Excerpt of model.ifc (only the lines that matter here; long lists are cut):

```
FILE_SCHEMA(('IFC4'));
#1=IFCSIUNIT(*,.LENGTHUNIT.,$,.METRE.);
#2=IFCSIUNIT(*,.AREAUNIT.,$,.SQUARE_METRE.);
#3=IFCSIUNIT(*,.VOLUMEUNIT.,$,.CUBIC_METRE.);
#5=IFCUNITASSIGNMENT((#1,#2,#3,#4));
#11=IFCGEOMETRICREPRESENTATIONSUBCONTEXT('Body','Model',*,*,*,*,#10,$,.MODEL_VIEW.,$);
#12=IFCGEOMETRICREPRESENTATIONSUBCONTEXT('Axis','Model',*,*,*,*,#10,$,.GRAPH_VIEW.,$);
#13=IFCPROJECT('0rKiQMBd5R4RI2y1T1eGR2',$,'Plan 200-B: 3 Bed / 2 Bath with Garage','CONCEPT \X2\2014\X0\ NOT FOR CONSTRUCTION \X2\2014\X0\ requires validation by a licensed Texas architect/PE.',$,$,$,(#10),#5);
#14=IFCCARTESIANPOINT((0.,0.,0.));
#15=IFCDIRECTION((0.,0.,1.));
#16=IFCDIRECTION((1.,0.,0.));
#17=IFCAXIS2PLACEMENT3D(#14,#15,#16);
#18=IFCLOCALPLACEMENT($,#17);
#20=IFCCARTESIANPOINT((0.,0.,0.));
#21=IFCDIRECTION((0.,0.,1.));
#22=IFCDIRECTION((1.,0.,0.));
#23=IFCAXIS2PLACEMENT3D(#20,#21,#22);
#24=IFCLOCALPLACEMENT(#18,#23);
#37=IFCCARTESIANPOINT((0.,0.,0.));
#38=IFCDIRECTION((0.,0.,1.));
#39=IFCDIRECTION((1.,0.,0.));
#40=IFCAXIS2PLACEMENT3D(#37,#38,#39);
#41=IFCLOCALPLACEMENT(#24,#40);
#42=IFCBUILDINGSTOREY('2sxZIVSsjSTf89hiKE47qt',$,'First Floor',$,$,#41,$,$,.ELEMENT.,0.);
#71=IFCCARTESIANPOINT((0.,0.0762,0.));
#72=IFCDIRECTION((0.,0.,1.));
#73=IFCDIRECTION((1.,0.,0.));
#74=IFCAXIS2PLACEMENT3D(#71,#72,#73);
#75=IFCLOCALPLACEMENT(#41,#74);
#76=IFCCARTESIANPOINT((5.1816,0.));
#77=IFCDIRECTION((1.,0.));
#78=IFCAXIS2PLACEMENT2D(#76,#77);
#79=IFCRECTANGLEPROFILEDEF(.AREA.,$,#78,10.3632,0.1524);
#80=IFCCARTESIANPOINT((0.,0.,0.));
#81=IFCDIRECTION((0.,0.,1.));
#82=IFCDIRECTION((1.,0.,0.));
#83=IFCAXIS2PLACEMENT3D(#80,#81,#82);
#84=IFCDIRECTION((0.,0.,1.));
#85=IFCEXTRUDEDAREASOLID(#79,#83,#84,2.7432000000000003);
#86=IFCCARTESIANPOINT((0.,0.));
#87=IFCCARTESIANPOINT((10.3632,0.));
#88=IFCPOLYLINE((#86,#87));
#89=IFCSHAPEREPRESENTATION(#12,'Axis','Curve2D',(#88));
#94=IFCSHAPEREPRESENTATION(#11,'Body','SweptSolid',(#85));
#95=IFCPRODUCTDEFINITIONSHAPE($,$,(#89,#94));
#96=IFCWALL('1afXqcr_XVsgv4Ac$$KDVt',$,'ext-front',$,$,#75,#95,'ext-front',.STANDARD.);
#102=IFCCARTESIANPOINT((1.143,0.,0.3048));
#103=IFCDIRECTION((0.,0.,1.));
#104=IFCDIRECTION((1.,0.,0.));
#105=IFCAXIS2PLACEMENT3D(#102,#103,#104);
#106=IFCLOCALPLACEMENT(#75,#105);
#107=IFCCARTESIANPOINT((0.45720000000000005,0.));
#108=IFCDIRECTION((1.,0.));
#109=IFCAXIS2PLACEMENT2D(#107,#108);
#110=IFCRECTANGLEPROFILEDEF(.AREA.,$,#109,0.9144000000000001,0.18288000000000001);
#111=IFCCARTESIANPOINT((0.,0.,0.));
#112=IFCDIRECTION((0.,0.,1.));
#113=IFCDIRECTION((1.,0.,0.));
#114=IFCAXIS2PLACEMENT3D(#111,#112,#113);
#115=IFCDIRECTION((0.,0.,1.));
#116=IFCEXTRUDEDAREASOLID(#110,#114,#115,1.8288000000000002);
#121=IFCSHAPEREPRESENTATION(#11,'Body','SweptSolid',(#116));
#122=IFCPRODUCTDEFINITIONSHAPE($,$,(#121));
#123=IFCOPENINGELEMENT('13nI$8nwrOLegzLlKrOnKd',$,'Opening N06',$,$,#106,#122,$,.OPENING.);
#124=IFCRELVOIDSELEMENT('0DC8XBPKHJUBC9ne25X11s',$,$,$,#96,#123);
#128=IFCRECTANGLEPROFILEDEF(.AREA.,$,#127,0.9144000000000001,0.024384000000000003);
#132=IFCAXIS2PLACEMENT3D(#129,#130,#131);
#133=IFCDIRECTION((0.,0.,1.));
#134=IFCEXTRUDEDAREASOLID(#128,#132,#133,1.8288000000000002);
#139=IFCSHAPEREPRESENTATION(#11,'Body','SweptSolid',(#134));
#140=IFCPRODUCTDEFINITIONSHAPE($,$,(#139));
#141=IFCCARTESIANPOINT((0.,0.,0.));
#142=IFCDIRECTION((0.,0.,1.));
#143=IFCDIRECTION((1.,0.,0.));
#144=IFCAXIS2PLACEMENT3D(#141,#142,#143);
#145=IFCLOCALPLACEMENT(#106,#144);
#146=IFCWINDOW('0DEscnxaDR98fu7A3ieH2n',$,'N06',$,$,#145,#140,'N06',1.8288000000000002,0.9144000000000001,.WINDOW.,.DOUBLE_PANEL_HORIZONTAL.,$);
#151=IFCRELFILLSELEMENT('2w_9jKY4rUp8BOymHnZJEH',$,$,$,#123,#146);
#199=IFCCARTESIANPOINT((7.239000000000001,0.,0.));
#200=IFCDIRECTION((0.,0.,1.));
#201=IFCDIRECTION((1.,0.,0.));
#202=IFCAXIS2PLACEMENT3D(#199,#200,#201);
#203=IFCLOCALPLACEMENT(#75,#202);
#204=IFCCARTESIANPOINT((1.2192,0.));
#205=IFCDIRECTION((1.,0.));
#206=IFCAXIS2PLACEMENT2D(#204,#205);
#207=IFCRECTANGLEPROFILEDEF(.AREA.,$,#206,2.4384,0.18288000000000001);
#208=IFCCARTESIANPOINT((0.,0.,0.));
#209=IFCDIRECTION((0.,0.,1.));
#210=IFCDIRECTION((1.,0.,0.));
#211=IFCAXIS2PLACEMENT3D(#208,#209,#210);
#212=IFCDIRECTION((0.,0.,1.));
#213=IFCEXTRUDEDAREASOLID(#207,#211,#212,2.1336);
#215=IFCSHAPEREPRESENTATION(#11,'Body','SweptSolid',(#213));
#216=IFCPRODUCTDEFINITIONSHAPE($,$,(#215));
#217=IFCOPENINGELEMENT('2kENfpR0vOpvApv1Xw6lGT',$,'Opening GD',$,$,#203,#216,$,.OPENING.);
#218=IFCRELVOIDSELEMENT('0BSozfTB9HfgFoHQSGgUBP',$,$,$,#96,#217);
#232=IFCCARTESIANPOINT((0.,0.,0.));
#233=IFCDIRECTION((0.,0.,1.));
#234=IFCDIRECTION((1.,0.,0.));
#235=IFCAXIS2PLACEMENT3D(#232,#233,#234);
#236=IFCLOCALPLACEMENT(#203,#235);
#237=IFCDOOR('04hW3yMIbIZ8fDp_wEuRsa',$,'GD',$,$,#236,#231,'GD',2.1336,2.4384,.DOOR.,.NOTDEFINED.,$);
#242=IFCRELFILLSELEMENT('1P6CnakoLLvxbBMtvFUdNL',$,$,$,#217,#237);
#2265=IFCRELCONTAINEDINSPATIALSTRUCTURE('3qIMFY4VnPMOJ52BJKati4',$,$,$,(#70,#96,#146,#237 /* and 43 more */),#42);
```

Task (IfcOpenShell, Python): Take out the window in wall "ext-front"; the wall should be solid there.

```python
import ifcopenshell
import ifcopenshell.api.feature
import ifcopenshell.api.root
import ifcopenshell.geom
import ifcopenshell.util.shape

model = ifcopenshell.open("model.ifc")
settings = ifcopenshell.geom.settings()


def volume(element):
    """Net volume in cubic metres, openings subtracted."""
    shape = ifcopenshell.geom.create_shape(settings, element)
    return ifcopenshell.util.shape.get_volume(shape.geometry)


window = model.by_guid("0DEscnxaDR98fu7A3ieH2n")
opening = window.FillsVoids[0].RelatingOpeningElement
wall = opening.VoidsElements[0].RelatingBuildingElement
before = volume(wall)

ifcopenshell.api.root.remove_product(model, product=window)
ifcopenshell.api.feature.remove_feature(model, feature=opening)

after = volume(wall)

print(f"wall volume {before:.3f} -> {after:.3f} m3")

model.write("model-out.ifc")
```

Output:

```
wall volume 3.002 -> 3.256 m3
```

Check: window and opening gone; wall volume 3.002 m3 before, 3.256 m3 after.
